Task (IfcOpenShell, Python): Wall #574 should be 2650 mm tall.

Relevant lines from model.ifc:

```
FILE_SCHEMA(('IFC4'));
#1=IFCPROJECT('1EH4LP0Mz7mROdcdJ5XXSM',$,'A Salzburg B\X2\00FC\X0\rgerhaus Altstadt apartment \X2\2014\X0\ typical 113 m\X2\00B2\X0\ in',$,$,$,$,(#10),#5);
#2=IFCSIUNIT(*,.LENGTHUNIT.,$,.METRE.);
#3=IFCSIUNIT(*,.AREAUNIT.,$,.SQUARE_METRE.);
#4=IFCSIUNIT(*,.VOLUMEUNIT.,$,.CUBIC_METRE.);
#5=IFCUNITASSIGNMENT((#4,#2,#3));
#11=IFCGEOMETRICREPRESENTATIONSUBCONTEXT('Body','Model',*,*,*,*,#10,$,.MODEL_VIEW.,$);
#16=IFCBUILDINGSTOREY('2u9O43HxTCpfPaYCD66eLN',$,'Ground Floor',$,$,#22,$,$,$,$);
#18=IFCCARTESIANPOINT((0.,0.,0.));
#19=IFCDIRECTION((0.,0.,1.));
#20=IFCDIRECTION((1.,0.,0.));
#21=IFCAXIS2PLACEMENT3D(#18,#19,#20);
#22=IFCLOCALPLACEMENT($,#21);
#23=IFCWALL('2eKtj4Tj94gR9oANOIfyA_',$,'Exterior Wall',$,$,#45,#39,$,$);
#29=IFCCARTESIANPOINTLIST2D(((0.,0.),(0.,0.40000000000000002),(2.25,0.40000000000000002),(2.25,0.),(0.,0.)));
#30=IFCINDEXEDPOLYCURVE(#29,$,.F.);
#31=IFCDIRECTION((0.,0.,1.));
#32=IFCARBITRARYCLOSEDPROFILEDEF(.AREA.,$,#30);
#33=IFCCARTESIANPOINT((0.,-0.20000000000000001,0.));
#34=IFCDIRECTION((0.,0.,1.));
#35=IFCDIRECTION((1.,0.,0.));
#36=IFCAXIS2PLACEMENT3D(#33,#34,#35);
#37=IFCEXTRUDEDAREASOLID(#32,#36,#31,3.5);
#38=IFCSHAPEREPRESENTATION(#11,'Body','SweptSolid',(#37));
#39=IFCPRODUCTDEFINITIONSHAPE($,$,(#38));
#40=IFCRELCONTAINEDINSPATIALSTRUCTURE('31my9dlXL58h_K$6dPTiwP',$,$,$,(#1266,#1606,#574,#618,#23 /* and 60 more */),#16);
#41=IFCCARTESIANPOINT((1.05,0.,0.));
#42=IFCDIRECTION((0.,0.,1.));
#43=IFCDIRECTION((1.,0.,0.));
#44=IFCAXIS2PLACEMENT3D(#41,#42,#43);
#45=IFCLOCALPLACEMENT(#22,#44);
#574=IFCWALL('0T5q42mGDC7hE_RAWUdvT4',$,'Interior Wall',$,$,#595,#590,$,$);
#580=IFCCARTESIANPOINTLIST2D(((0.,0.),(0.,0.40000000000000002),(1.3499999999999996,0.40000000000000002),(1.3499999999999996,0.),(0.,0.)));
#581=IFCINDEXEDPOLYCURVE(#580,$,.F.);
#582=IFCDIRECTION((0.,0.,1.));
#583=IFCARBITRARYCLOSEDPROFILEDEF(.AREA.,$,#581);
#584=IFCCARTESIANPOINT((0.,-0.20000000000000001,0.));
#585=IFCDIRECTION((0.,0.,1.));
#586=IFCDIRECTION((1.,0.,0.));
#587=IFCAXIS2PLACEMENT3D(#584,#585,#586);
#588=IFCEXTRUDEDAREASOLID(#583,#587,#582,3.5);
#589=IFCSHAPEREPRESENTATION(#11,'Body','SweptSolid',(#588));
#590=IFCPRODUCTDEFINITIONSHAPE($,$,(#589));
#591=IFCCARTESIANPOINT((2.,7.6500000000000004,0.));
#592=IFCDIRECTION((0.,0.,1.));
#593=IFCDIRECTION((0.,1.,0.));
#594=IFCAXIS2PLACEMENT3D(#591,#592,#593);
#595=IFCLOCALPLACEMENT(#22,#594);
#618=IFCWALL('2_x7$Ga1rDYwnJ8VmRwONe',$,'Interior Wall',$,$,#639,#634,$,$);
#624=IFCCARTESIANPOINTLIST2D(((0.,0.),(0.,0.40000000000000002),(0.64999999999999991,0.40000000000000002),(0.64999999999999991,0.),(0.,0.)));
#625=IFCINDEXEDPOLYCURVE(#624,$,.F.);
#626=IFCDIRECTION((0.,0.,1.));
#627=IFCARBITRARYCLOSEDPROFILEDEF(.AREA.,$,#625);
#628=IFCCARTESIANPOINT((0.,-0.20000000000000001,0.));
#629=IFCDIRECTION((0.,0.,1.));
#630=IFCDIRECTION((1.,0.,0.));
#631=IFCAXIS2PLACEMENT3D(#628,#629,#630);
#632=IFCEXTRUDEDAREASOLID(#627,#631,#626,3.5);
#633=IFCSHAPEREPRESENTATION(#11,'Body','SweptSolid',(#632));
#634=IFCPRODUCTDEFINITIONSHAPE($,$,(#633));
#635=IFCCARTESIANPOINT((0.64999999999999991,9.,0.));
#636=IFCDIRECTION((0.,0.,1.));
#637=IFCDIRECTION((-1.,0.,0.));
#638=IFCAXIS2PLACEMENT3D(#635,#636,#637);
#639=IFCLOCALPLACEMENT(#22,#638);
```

```python
import ifcopenshell
import ifcopenshell.geom
import ifcopenshell.util.representation
import ifcopenshell.util.shape

model = ifcopenshell.open("model.ifc")
settings = ifcopenshell.geom.settings()


def volume(element):
    """Net volume in cubic metres, openings subtracted."""
    shape = ifcopenshell.geom.create_shape(settings, element)
    return ifcopenshell.util.shape.get_volume(shape.geometry)


wall = model.by_id(574)
before = volume(wall)

body = ifcopenshell.util.representation.get_representation(wall, "Model", "Body")
solid = body.Items[0]
old_height = solid.Depth
solid.Depth = 2.65
after = volume(wall)

print(f"height {old_height:g} -> {solid.Depth:g}, volume {before:.3f} -> {after:.3f} m3")

model.write("model-out.ifc")
```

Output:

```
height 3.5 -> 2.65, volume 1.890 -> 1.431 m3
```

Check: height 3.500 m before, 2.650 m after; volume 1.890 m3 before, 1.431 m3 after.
